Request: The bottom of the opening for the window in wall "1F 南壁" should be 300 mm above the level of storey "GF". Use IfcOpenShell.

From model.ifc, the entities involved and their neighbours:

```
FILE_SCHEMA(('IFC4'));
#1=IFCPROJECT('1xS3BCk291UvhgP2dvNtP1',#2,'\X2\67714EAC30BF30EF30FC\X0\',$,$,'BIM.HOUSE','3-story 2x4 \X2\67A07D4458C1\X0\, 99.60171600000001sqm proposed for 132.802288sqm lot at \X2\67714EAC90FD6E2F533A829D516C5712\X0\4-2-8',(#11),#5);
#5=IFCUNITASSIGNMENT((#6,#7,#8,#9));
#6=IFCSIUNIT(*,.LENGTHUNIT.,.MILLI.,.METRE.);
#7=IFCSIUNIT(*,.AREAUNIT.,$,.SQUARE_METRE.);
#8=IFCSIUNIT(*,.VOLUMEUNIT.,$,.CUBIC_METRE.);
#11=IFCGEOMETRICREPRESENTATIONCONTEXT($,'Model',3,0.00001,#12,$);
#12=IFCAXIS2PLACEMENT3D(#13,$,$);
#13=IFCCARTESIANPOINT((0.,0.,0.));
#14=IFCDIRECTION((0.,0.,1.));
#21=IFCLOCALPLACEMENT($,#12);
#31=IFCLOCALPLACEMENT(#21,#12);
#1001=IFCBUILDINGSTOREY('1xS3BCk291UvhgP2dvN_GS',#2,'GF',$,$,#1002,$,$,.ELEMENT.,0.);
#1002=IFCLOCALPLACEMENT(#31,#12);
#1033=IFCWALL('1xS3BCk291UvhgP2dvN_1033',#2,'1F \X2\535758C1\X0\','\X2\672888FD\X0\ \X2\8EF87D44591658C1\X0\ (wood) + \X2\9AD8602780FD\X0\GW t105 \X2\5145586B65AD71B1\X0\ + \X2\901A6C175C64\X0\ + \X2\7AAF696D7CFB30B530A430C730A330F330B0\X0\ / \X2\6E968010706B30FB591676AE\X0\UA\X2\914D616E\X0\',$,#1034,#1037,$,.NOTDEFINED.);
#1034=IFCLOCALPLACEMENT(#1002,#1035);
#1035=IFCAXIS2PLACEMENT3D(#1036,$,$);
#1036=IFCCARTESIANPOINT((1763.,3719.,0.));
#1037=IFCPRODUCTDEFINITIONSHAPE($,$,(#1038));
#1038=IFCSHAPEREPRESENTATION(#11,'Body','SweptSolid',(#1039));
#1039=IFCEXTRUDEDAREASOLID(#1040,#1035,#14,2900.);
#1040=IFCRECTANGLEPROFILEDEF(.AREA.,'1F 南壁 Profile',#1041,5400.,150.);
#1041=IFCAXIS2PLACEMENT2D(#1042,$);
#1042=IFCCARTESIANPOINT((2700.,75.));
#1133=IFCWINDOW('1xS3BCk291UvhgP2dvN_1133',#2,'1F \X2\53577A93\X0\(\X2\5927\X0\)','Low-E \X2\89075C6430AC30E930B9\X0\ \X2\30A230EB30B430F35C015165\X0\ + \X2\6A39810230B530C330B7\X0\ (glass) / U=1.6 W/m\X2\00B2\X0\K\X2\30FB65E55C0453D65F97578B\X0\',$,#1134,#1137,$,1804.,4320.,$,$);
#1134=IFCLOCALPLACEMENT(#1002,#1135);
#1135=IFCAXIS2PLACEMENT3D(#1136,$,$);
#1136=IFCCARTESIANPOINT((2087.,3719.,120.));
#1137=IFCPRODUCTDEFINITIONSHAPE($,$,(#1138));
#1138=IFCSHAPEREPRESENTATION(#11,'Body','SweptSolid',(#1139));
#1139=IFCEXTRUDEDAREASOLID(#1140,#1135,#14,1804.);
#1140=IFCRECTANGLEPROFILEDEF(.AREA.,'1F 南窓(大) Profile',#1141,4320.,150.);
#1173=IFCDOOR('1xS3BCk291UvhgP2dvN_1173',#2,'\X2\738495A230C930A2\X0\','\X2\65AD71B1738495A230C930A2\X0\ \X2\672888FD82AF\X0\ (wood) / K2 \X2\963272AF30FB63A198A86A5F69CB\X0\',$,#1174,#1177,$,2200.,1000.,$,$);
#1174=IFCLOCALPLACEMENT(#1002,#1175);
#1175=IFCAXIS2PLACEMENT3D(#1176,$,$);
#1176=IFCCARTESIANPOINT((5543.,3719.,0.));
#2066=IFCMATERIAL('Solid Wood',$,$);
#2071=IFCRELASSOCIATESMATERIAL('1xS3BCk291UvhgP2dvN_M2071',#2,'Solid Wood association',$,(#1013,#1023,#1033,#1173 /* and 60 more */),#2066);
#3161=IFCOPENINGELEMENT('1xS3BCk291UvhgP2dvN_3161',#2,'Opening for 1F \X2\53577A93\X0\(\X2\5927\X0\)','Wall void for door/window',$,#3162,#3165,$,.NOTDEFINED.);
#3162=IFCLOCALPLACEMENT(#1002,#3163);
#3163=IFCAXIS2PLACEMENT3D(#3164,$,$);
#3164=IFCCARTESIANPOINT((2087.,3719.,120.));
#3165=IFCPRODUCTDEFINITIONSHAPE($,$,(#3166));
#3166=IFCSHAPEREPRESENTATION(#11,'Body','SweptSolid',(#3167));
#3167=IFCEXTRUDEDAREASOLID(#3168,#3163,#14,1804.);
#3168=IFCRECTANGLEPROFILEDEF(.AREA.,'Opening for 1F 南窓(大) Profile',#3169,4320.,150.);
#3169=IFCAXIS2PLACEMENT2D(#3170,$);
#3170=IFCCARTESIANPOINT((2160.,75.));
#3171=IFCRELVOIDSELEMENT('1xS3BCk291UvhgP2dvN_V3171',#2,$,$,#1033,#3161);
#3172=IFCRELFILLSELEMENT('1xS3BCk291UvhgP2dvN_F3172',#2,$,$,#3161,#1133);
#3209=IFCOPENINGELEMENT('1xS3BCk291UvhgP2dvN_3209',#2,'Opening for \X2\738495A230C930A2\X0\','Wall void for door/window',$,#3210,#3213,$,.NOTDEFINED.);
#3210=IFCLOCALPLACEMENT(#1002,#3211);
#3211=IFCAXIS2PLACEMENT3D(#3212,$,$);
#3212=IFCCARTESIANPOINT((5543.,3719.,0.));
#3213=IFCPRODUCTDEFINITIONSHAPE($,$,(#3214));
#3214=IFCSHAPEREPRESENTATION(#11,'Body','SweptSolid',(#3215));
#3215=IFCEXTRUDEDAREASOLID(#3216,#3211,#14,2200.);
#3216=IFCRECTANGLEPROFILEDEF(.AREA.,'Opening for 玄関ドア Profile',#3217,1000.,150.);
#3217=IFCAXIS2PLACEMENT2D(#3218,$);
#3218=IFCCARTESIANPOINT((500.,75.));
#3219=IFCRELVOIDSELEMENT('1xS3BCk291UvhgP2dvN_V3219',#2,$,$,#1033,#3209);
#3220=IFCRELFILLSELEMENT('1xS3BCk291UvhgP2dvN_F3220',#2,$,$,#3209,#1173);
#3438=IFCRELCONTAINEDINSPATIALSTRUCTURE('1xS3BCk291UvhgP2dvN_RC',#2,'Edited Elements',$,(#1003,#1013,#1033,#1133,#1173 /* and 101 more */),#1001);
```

```python
import numpy as np
import ifcopenshell
import ifcopenshell.api.geometry
import ifcopenshell.geom
import ifcopenshell.util.element
import ifcopenshell.util.placement
import ifcopenshell.util.shape
import ifcopenshell.util.unit

model = ifcopenshell.open("model.ifc")
unit_scale = ifcopenshell.util.unit.calculate_unit_scale(model)

window = model.by_guid("1xS3BCk291UvhgP2dvN_1133")
opening = window.FillsVoids[0].RelatingOpeningElement
storey = ifcopenshell.util.element.get_container(window, ifc_class="IfcBuildingStorey")
level = ifcopenshell.util.placement.get_local_placement(storey.ObjectPlacement)[2, 3]

# The opening's origin need not be at the sill, so measure its lowest point.
shape = ifcopenshell.geom.create_shape(ifcopenshell.geom.settings(), opening)
bottom = ifcopenshell.util.shape.get_shape_bottom_elevation(shape, shape.geometry) / unit_scale
dz = level + 0.3 / unit_scale - bottom

shift = np.array([0.0, 0.0, dz])
# The window is not placed relative to its opening, so move both.
for product in (opening, window):
    matrix = ifcopenshell.util.placement.get_local_placement(product.ObjectPlacement)
    matrix[:3, 3] += shift
    ifcopenshell.api.geometry.edit_object_placement(model, product=product, matrix=matrix, is_si=False)

print(f"moved by {dz * unit_scale:+.3f} m")

model.write("model_v2.ifc")
```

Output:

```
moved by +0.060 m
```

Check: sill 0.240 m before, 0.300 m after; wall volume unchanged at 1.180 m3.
